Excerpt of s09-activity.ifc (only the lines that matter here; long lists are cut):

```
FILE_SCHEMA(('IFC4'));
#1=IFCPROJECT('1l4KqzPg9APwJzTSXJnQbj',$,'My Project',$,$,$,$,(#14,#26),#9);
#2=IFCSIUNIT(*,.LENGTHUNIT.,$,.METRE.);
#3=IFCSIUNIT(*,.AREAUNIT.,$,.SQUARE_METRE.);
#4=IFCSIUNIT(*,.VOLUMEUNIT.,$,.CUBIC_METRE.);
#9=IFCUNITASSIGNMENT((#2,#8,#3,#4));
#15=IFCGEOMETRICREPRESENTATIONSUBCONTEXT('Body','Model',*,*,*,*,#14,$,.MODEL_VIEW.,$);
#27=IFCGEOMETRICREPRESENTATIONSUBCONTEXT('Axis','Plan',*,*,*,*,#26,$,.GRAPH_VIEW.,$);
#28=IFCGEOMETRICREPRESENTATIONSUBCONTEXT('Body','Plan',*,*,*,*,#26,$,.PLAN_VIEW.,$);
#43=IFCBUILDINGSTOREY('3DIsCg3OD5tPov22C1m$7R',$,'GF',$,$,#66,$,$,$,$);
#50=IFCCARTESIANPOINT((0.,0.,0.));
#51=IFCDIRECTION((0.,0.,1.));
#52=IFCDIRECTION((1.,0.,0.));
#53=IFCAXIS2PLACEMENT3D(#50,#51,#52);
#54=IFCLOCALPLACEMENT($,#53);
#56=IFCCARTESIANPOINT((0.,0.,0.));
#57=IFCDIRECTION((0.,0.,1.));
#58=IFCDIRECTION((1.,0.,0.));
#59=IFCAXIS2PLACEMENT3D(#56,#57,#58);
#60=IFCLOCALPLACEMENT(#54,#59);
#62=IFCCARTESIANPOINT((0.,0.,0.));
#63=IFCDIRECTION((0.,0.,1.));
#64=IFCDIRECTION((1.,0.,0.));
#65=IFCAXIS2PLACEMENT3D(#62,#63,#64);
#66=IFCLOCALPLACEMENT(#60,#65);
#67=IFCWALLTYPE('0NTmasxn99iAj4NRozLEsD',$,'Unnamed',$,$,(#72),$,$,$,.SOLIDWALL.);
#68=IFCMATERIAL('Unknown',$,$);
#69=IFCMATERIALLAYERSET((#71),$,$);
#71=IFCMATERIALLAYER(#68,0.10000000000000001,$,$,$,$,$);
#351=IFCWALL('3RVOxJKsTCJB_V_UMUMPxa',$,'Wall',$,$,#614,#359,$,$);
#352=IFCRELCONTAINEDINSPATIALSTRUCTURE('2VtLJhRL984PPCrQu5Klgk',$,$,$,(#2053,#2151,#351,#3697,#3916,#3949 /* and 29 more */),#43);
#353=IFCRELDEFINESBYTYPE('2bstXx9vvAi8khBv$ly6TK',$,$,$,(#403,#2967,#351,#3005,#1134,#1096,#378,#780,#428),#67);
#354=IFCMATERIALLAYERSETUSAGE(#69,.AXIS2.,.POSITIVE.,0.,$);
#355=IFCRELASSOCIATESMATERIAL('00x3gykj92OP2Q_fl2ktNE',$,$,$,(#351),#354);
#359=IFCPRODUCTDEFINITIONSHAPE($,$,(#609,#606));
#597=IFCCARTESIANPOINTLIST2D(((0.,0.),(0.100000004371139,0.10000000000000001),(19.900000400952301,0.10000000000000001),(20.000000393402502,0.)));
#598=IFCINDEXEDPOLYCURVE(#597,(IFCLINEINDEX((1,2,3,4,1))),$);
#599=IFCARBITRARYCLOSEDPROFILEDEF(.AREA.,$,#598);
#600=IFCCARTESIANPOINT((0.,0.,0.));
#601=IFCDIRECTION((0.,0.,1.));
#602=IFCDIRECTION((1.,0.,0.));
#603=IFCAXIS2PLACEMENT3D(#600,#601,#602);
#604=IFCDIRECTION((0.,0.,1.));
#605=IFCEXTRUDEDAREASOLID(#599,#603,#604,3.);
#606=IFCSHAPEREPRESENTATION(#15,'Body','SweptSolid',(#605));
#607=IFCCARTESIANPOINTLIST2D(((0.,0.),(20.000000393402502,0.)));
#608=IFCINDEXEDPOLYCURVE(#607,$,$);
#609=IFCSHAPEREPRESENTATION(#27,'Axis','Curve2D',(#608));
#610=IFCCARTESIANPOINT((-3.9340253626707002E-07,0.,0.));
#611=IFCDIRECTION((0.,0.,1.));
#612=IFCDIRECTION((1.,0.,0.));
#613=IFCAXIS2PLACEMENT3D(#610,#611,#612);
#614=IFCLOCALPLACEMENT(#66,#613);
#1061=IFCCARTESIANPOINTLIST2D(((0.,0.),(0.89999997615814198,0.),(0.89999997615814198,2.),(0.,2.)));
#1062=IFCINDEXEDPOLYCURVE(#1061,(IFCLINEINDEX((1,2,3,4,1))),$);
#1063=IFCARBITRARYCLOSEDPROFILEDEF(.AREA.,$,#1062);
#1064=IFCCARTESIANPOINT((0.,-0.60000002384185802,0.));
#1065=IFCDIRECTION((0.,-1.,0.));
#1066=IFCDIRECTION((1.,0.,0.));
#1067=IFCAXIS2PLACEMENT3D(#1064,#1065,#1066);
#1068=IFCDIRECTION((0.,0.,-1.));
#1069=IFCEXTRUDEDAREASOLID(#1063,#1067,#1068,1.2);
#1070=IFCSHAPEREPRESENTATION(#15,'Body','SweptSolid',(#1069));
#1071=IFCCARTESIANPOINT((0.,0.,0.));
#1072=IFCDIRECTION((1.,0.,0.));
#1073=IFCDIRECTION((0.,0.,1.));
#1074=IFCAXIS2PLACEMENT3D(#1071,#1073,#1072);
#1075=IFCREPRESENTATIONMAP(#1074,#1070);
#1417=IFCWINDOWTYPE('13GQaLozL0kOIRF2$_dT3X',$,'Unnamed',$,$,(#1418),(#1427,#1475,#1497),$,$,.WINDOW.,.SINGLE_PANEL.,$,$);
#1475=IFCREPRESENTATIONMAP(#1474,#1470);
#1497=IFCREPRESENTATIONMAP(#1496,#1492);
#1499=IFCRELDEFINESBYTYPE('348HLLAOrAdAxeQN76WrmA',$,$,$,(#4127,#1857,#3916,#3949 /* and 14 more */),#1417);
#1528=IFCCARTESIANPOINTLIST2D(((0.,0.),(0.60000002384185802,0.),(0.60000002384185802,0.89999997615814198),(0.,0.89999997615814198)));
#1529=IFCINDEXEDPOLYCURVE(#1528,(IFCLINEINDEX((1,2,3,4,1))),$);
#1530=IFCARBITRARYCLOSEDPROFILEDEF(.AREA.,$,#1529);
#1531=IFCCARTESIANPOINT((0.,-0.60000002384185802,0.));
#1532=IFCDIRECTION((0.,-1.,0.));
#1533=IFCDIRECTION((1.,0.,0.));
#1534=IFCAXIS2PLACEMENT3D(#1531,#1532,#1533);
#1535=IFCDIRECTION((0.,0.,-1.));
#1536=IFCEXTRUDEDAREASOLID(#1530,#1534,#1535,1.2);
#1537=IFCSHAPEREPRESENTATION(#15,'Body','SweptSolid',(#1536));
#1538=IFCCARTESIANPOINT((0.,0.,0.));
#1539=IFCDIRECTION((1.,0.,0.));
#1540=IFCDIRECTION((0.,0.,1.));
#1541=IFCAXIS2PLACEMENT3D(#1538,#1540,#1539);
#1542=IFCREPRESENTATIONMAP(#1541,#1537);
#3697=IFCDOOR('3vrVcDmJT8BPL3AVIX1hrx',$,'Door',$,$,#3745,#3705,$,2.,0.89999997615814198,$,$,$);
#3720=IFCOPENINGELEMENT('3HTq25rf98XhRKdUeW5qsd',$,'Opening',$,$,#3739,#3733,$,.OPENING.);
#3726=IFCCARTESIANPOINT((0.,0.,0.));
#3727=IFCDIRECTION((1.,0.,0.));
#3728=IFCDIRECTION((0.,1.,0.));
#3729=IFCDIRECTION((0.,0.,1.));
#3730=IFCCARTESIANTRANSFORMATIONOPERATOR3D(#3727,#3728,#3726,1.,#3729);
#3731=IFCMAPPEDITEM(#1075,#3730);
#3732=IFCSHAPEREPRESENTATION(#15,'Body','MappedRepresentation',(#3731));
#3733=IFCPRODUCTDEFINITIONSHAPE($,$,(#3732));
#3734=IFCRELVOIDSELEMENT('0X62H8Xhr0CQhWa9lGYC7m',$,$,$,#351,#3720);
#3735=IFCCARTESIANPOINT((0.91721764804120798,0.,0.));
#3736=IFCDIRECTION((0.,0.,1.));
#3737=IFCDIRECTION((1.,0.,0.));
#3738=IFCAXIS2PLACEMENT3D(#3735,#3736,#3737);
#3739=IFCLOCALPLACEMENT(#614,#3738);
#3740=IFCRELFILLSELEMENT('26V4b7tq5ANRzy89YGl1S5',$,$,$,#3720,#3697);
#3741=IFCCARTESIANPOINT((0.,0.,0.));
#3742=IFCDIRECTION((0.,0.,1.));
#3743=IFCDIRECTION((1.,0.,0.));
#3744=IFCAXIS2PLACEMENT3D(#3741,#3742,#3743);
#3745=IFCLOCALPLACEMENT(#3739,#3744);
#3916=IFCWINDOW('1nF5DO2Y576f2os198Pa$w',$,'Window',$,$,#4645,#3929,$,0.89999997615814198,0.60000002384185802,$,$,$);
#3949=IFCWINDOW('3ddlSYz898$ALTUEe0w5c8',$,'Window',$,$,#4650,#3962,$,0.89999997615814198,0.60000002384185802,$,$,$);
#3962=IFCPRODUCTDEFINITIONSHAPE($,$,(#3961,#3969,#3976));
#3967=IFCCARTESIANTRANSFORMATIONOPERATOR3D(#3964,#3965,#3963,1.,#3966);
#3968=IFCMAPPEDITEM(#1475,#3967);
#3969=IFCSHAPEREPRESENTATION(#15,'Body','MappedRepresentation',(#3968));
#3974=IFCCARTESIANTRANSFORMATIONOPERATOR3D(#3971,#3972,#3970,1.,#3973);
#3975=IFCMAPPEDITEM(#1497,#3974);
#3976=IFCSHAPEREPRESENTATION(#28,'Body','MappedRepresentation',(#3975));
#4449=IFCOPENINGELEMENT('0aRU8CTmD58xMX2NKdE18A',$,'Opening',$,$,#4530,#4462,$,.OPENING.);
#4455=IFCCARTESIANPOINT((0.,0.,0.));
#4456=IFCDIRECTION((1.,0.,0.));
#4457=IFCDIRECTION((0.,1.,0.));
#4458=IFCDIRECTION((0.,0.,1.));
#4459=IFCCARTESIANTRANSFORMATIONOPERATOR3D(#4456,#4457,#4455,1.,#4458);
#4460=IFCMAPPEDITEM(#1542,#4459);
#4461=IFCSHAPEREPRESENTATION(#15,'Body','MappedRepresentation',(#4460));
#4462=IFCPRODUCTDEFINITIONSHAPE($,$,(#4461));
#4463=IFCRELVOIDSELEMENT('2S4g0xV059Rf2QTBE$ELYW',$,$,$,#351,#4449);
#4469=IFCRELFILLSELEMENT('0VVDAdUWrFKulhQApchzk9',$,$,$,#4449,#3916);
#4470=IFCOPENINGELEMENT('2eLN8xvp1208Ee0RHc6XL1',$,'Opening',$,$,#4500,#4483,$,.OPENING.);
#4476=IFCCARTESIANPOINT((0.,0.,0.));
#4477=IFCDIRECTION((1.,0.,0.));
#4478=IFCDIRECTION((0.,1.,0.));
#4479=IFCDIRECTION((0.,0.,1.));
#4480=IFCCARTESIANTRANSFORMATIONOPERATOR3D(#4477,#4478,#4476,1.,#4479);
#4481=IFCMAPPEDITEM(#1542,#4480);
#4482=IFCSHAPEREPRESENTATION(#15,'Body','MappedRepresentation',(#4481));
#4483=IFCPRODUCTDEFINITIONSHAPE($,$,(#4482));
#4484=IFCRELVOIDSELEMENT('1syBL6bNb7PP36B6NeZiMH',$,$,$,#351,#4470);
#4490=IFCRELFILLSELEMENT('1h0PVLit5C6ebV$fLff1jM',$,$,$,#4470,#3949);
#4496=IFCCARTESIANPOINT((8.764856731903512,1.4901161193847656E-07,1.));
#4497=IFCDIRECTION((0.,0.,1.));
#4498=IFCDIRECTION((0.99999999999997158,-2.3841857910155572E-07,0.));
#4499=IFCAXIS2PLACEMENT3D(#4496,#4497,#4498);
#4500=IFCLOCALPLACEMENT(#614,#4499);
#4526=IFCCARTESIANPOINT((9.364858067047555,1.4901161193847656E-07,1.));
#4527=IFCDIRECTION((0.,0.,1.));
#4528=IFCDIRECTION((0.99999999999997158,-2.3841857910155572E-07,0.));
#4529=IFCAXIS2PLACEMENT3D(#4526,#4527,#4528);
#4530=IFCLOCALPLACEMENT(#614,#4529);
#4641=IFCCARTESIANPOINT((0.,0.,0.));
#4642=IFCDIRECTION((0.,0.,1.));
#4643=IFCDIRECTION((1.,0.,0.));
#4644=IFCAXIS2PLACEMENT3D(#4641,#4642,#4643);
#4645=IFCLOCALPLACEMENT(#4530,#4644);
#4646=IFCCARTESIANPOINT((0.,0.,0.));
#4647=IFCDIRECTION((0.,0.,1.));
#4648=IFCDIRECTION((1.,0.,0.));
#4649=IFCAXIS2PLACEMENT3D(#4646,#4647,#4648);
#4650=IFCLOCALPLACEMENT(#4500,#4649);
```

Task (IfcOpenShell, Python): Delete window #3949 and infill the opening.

```python
import ifcopenshell
import ifcopenshell.api.feature
import ifcopenshell.api.root
import ifcopenshell.geom
import ifcopenshell.util.shape

model = ifcopenshell.open("s09-activity.ifc")
settings = ifcopenshell.geom.settings()


def volume(element):
    """Net volume in cubic metres, openings subtracted."""
    shape = ifcopenshell.geom.create_shape(settings, element)
    return ifcopenshell.util.shape.get_volume(shape.geometry)


window = model.by_guid("3ddlSYz898$ALTUEe0w5c8")
opening = window.FillsVoids[0].RelatingOpeningElement
wall = opening.VoidsElements[0].RelatingBuildingElement
before = volume(wall)

ifcopenshell.api.root.remove_product(model, product=window)
ifcopenshell.api.feature.remove_feature(model, feature=opening)

after = volume(wall)

print(f"wall volume {before:.3f} -> {after:.3f} m3")

model.write("s09-activity_edited.ifc")
```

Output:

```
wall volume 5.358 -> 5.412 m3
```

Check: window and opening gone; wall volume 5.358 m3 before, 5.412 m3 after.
